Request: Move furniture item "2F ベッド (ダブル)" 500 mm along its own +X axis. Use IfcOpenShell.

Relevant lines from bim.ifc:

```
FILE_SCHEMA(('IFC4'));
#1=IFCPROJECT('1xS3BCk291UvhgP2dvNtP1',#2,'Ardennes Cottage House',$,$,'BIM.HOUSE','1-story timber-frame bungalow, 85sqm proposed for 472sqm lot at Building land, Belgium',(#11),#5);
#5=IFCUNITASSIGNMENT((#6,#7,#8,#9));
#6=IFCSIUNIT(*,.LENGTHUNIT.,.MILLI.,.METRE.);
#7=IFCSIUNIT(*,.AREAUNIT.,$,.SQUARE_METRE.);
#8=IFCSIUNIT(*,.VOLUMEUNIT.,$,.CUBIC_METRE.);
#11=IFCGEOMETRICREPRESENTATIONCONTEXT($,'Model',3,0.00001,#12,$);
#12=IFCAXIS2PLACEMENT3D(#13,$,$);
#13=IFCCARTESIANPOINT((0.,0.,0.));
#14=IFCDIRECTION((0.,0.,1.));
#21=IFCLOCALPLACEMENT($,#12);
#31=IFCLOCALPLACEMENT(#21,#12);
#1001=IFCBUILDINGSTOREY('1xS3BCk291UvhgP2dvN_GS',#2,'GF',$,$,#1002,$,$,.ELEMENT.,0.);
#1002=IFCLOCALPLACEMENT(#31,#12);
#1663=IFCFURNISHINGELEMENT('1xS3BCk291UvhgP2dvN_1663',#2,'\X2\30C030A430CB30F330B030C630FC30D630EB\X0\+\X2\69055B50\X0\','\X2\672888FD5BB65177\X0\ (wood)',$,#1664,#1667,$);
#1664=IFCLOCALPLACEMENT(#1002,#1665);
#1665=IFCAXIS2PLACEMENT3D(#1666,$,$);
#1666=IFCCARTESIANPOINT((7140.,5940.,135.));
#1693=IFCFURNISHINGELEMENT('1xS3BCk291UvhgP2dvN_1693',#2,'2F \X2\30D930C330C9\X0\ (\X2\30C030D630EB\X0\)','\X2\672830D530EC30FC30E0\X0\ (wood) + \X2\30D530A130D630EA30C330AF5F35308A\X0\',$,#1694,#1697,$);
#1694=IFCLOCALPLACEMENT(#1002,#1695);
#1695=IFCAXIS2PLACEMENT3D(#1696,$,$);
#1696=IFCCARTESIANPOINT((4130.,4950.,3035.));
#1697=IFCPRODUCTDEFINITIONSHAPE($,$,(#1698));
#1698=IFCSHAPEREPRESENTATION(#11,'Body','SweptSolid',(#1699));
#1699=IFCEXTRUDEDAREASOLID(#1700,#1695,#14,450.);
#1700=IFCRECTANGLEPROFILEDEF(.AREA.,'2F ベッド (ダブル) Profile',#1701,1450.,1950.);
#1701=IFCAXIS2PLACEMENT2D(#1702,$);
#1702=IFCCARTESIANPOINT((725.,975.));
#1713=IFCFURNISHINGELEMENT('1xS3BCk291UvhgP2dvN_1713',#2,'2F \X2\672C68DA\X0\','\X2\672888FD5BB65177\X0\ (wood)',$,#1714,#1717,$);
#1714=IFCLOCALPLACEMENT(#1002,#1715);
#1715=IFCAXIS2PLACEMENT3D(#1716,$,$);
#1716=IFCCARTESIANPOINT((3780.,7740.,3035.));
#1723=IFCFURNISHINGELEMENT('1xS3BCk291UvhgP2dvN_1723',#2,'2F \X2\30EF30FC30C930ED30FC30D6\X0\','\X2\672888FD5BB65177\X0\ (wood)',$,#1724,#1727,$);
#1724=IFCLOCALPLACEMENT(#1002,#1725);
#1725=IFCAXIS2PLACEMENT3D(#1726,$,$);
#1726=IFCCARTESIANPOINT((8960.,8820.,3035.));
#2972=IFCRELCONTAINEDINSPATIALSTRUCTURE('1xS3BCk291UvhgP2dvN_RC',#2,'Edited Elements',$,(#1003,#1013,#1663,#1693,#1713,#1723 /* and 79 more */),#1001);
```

```python
import ifcopenshell
import ifcopenshell.api.geometry
import ifcopenshell.util.placement
import ifcopenshell.util.unit

model = ifcopenshell.open("bim.ifc")
unit_scale = ifcopenshell.util.unit.calculate_unit_scale(model)

item = model.by_guid("1xS3BCk291UvhgP2dvN_1693")
matrix = ifcopenshell.util.placement.get_local_placement(item.ObjectPlacement)
matrix[:3, 3] += matrix[:3, 0] * 0.5 / unit_scale
ifcopenshell.api.geometry.edit_object_placement(model, product=item, matrix=matrix, is_si=False)

print(ifcopenshell.util.placement.get_local_placement(item.ObjectPlacement).round(3) + 0.0)

model.write("bim_edited.ifc")
```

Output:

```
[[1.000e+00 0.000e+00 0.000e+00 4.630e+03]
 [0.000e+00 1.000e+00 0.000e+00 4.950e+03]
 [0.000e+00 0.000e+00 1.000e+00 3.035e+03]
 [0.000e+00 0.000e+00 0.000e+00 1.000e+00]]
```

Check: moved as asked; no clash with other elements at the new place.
